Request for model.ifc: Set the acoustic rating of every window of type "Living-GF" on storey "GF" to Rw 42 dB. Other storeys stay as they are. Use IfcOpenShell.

First a look at what the model holds.

```python
import ifcopenshell
import ifcopenshell.util.element

model = ifcopenshell.open("model.ifc")
print(model.schema)
storey = next(s for s in model.by_type("IfcBuildingStorey") if s.Name == "GF")
windows = [e for e in ifcopenshell.util.element.get_decomposition(storey) if e.is_a("IfcWindow")]
seen = {}
for e in windows:
    element_type = ifcopenshell.util.element.get_type(e)
    key = (element_type.Name if element_type != e and element_type else None, ifcopenshell.util.element.get_pset(e, "Pset_WindowCommon", "AcousticRating"))
    seen[key] = seen.get(key, 0) + 1
for (name, value), count in sorted(seen.items(), key=str):
    print(count, "x", name, "|", value)
```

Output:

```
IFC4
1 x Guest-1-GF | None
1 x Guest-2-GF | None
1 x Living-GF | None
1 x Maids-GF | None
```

```python
import ifcopenshell
import ifcopenshell.api.pset
import ifcopenshell.util.element

model = ifcopenshell.open("model.ifc")

storey = next(s for s in model.by_type("IfcBuildingStorey") if s.Name == "GF")
windows = [e for e in ifcopenshell.util.element.get_decomposition(storey) if e.is_a("IfcWindow")]

count = 0
for e in windows:
    element_type = ifcopenshell.util.element.get_type(e)
    if element_type in (None, e) or element_type.Name != "Living-GF":
        continue
    # add_pset returns the element's existing set when there is one.
    pset = ifcopenshell.api.pset.add_pset(model, product=e, name="Pset_WindowCommon")
    ifcopenshell.api.pset.edit_pset(model, pset=pset, properties={"AcousticRating": "Rw 42 dB"})
    count += 1

print(count, "windows updated")

model.write("model_rev.ifc")
```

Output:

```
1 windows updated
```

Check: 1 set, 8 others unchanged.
